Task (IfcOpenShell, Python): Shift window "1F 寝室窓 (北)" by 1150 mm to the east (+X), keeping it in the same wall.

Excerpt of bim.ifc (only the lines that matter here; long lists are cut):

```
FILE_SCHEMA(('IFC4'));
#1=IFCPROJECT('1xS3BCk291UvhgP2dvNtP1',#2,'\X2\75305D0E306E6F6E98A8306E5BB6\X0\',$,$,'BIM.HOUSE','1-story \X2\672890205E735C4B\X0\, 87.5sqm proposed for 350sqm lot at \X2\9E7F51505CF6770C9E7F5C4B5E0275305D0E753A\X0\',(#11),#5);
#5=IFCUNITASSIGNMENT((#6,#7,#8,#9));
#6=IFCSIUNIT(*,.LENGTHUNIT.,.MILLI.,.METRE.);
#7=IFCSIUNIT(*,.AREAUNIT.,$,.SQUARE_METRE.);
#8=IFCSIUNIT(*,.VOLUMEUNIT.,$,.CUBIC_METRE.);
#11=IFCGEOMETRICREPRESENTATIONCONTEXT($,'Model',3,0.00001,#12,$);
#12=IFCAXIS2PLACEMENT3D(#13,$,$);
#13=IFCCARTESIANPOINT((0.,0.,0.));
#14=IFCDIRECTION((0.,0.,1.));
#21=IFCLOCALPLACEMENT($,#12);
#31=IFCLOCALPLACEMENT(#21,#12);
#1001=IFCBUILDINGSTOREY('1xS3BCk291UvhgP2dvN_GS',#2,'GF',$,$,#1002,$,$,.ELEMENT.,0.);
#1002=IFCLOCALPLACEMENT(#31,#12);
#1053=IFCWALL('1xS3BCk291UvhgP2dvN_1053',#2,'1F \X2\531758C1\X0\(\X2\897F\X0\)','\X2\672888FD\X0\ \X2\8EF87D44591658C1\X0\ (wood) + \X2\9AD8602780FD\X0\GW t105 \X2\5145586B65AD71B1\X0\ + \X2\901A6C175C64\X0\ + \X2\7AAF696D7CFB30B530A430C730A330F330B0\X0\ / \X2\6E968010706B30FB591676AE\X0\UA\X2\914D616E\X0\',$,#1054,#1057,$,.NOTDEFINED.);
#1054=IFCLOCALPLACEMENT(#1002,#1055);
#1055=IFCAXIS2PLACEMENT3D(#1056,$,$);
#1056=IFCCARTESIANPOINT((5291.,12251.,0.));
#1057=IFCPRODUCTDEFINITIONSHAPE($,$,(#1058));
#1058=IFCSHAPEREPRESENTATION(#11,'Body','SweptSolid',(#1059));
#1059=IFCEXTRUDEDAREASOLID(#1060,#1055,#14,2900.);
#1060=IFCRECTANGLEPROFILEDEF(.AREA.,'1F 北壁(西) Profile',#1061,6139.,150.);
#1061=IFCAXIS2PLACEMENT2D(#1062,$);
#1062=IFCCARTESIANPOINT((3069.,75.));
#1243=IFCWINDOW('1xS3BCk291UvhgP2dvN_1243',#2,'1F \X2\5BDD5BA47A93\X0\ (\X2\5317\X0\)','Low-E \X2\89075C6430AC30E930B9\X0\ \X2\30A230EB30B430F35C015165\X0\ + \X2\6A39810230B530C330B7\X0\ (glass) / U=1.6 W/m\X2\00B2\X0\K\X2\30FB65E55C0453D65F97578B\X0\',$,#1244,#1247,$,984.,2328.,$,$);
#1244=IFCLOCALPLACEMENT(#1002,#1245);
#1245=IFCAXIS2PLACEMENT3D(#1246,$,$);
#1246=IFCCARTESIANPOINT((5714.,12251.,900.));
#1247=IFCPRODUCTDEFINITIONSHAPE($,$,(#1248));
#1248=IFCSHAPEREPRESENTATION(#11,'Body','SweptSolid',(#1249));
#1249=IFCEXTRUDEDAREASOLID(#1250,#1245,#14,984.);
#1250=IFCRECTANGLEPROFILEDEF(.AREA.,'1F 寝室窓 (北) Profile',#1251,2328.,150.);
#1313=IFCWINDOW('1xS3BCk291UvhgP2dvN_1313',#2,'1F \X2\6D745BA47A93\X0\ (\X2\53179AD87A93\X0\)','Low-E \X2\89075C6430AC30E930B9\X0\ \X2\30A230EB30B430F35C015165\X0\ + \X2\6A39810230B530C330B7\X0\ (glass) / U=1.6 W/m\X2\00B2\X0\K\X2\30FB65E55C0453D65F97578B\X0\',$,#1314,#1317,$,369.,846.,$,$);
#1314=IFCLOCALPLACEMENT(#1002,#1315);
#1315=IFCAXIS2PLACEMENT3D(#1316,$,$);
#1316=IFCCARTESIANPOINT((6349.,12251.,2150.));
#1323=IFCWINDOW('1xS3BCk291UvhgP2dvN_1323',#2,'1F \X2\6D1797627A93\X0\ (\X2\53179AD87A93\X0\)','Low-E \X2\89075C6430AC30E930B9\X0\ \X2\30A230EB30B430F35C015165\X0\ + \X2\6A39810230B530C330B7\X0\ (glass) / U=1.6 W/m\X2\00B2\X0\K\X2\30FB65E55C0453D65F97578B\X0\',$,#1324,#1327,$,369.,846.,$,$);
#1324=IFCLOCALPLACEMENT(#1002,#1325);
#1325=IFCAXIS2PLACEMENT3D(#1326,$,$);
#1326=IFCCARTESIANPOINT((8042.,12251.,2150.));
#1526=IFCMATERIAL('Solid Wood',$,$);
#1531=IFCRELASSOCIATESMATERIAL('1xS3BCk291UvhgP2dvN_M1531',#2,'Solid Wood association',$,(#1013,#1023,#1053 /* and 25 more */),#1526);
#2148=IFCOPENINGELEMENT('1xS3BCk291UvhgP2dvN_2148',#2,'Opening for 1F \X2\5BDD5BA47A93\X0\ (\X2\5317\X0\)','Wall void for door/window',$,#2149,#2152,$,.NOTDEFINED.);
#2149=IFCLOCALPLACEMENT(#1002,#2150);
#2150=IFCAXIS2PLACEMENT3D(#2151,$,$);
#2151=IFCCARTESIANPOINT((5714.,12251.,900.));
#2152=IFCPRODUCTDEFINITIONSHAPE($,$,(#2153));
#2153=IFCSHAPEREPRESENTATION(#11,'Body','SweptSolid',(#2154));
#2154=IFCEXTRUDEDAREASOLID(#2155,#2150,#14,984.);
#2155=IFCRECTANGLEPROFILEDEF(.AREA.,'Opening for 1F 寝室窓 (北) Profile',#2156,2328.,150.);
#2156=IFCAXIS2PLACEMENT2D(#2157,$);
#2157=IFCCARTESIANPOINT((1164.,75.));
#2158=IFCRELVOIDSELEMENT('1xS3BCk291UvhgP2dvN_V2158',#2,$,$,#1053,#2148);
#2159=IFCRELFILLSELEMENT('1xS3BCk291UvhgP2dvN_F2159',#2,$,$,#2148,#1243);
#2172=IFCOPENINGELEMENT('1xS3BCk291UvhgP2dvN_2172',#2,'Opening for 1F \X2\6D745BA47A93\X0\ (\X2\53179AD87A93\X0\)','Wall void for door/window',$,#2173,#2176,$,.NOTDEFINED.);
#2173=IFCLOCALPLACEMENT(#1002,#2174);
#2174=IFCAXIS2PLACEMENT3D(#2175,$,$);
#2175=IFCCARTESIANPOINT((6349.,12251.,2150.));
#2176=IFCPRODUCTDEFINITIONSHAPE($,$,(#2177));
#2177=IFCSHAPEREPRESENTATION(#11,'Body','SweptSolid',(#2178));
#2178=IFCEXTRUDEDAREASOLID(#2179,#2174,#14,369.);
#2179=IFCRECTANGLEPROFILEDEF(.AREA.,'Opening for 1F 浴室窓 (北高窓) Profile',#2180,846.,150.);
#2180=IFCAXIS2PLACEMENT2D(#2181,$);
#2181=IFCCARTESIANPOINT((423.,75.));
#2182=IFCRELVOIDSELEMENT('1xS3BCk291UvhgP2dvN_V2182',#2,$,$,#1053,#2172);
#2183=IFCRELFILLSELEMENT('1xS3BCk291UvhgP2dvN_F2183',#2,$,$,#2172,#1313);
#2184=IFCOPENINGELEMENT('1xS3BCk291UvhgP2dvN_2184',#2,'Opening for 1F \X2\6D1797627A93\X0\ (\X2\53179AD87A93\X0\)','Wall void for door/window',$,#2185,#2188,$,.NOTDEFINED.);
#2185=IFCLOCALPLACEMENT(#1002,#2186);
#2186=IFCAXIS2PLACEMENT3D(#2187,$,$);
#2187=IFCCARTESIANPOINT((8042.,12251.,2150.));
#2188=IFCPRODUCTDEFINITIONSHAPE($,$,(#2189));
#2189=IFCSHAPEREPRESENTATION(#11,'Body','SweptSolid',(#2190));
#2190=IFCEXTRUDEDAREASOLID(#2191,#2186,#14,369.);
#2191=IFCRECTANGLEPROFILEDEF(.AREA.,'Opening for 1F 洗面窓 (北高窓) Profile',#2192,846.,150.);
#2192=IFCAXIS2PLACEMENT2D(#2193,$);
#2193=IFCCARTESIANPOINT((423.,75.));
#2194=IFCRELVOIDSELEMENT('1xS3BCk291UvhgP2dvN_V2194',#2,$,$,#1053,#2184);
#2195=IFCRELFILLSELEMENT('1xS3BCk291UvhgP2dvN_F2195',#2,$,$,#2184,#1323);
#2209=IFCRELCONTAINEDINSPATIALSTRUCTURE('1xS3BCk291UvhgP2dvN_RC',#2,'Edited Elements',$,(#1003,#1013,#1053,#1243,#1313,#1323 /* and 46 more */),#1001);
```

```python
import ifcopenshell
import ifcopenshell.api.geometry
import ifcopenshell.util.placement

model = ifcopenshell.open("bim.ifc")

window = model.by_guid("1xS3BCk291UvhgP2dvN_1243")
opening = window.FillsVoids[0].RelatingOpeningElement
wall = opening.VoidsElements[0].RelatingBuildingElement

wall_matrix = ifcopenshell.util.placement.get_local_placement(wall.ObjectPlacement)
shift = wall_matrix[:3, 0] * 1150.0
before = ifcopenshell.util.placement.get_local_placement(window.ObjectPlacement)[:3, 3].copy()

# The window is not placed relative to its opening, so move both.
for product in (opening, window):
    matrix = ifcopenshell.util.placement.get_local_placement(product.ObjectPlacement)
    matrix[:3, 3] += shift
    ifcopenshell.api.geometry.edit_object_placement(model, product=product, matrix=matrix, is_si=False)

after = ifcopenshell.util.placement.get_local_placement(window.ObjectPlacement)[:3, 3]
print("window moved by", (after - before).round(3) + 0.0)

model.write("bim_v2.ifc")
```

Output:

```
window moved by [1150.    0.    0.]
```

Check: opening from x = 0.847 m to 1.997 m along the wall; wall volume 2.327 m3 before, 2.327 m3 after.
